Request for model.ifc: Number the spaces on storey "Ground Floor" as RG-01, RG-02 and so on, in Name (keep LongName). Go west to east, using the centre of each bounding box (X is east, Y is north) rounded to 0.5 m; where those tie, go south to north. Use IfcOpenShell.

First a look at what the model holds.

```python
import ifcopenshell
import ifcopenshell.util.element
import ifcopenshell.util.placement

model = ifcopenshell.open("model.ifc")
print(model.schema)
storey = next(s for s in model.by_type("IfcBuildingStorey") if s.Name == "Ground Floor")
spaces = [e for e in ifcopenshell.util.element.get_decomposition(storey) if e.is_a("IfcSpace")]
for e in sorted(spaces, key=lambda e: e.id()):
    origin = ifcopenshell.util.placement.get_local_placement(e.ObjectPlacement)[:3, 3]
    print(e.id(), e.Name, e.LongName, origin.round(2) + 0.0, sep=" | ")
```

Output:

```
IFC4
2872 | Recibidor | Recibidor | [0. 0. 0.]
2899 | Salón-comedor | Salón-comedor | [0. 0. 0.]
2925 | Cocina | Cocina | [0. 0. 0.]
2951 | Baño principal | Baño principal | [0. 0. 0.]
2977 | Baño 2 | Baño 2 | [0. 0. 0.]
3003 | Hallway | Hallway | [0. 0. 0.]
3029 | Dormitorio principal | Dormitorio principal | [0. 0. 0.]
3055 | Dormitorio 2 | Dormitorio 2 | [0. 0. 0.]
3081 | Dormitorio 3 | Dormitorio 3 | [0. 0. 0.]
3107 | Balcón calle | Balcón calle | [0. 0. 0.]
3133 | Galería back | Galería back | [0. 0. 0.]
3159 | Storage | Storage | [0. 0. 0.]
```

```python
import ifcopenshell
import ifcopenshell.geom
import ifcopenshell.util.element
import ifcopenshell.util.shape

model = ifcopenshell.open("model.ifc")
settings = ifcopenshell.geom.settings()
settings.set("use-world-coords", True)


def centre(element):
    shape = ifcopenshell.geom.create_shape(settings, element)
    return ifcopenshell.util.shape.get_bbox_centroid(shape.geometry)


storey = next(s for s in model.by_type("IfcBuildingStorey") if s.Name == "Ground Floor")
spaces = [e for e in ifcopenshell.util.element.get_decomposition(storey) if e.is_a("IfcSpace")]

# Insertion points can sit at a corner or the storey origin, so sort by the geometry (in metres).
centres = {e: centre(e) for e in spaces}
spaces.sort(key=lambda e: (round(centres[e][0] / 0.5), centres[e][1]))

for i, e in enumerate(spaces, start=1):
    number = f"RG-{i:02d}"
    e.Name = number
    print(e.id(), number)

model.write("model-out.ifc")
```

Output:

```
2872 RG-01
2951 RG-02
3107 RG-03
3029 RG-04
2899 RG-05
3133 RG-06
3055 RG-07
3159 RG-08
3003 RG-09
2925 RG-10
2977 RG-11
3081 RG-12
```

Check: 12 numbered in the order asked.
